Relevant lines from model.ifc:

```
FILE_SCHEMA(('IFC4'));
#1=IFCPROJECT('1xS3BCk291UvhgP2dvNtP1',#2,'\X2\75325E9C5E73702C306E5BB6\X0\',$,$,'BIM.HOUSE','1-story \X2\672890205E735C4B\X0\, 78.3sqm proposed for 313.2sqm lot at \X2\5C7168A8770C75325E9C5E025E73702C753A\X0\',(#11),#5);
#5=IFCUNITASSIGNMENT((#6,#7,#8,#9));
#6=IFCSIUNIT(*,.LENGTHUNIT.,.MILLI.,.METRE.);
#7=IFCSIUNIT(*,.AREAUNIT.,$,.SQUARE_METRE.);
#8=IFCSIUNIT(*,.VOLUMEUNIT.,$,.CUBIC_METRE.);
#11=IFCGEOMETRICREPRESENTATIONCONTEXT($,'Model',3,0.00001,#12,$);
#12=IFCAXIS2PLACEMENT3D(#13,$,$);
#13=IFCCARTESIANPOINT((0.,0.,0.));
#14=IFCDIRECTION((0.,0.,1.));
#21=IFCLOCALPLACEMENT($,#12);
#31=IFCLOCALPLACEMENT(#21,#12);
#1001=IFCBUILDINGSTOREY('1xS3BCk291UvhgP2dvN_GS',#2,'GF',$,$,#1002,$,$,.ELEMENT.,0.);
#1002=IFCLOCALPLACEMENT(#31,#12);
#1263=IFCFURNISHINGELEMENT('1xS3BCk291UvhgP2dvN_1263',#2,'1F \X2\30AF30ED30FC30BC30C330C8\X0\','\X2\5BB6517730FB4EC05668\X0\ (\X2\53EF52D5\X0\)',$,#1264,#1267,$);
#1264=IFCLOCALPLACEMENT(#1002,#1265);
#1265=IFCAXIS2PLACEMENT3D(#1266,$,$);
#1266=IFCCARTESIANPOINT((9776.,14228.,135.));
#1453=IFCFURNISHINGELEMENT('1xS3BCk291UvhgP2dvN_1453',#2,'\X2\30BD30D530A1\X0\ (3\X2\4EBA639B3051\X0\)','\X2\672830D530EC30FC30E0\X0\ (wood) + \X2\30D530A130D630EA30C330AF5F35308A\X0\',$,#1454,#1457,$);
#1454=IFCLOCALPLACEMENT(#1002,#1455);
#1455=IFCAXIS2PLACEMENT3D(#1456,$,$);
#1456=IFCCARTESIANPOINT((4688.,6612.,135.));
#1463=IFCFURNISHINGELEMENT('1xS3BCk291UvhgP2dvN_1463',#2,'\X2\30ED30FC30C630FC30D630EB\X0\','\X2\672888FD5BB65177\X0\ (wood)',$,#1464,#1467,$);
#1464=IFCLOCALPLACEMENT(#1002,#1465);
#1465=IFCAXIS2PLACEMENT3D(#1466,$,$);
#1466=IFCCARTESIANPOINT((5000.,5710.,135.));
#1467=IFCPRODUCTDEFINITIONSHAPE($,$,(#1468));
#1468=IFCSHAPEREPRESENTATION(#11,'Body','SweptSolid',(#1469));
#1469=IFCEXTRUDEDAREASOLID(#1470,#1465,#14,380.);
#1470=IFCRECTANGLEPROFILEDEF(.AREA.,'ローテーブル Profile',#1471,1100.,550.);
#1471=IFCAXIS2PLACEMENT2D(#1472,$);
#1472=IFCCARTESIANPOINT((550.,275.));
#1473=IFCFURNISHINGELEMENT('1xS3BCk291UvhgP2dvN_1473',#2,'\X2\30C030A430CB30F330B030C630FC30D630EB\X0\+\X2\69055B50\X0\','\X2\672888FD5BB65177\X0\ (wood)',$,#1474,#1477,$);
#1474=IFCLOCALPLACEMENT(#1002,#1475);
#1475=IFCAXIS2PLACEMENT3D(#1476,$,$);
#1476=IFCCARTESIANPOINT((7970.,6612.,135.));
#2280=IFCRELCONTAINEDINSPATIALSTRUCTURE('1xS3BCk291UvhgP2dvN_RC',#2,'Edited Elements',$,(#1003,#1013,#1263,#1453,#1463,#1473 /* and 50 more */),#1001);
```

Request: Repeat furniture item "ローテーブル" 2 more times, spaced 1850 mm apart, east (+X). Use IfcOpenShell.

```python
import numpy as np
import ifcopenshell
import ifcopenshell.api.geometry
import ifcopenshell.api.root
import ifcopenshell.util.element
import ifcopenshell.util.placement

model = ifcopenshell.open("model.ifc")


def reuse_history(source, copy):
    """copy_class also copies each property set's owner history, people and application; keep the originals."""
    for rel in copy.IsDefinedBy:
        if rel.is_a("IfcRelDefinesByProperties") and (history := rel.RelatingPropertyDefinition.OwnerHistory):
            rel.RelatingPropertyDefinition.OwnerHistory = source.OwnerHistory
            ifcopenshell.util.element.remove_deep2(model, history)


source = model.by_guid("1xS3BCk291UvhgP2dvN_1463")
base = ifcopenshell.util.placement.get_local_placement(source.ObjectPlacement)
step = np.array([1.0, 0.0, 0.0]) * 1850.0

for i in range(1, 3):
    copy = ifcopenshell.api.root.copy_class(model, product=source)
    copy.Representation = ifcopenshell.util.element.copy_deep(
        model, source.Representation, exclude=["IfcGeometricRepresentationContext", "IfcRepresentationMap"]
    )
    reuse_history(source, copy)
    matrix = base.copy()
    matrix[:3, 3] += i * step
    print("added at", matrix[:3, 3].round(3) + 0.0)
    ifcopenshell.api.geometry.edit_object_placement(model, product=copy, matrix=matrix, is_si=False)

model.write("model-out.ifc")
```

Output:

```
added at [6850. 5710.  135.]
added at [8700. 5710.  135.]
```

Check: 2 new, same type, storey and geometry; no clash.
